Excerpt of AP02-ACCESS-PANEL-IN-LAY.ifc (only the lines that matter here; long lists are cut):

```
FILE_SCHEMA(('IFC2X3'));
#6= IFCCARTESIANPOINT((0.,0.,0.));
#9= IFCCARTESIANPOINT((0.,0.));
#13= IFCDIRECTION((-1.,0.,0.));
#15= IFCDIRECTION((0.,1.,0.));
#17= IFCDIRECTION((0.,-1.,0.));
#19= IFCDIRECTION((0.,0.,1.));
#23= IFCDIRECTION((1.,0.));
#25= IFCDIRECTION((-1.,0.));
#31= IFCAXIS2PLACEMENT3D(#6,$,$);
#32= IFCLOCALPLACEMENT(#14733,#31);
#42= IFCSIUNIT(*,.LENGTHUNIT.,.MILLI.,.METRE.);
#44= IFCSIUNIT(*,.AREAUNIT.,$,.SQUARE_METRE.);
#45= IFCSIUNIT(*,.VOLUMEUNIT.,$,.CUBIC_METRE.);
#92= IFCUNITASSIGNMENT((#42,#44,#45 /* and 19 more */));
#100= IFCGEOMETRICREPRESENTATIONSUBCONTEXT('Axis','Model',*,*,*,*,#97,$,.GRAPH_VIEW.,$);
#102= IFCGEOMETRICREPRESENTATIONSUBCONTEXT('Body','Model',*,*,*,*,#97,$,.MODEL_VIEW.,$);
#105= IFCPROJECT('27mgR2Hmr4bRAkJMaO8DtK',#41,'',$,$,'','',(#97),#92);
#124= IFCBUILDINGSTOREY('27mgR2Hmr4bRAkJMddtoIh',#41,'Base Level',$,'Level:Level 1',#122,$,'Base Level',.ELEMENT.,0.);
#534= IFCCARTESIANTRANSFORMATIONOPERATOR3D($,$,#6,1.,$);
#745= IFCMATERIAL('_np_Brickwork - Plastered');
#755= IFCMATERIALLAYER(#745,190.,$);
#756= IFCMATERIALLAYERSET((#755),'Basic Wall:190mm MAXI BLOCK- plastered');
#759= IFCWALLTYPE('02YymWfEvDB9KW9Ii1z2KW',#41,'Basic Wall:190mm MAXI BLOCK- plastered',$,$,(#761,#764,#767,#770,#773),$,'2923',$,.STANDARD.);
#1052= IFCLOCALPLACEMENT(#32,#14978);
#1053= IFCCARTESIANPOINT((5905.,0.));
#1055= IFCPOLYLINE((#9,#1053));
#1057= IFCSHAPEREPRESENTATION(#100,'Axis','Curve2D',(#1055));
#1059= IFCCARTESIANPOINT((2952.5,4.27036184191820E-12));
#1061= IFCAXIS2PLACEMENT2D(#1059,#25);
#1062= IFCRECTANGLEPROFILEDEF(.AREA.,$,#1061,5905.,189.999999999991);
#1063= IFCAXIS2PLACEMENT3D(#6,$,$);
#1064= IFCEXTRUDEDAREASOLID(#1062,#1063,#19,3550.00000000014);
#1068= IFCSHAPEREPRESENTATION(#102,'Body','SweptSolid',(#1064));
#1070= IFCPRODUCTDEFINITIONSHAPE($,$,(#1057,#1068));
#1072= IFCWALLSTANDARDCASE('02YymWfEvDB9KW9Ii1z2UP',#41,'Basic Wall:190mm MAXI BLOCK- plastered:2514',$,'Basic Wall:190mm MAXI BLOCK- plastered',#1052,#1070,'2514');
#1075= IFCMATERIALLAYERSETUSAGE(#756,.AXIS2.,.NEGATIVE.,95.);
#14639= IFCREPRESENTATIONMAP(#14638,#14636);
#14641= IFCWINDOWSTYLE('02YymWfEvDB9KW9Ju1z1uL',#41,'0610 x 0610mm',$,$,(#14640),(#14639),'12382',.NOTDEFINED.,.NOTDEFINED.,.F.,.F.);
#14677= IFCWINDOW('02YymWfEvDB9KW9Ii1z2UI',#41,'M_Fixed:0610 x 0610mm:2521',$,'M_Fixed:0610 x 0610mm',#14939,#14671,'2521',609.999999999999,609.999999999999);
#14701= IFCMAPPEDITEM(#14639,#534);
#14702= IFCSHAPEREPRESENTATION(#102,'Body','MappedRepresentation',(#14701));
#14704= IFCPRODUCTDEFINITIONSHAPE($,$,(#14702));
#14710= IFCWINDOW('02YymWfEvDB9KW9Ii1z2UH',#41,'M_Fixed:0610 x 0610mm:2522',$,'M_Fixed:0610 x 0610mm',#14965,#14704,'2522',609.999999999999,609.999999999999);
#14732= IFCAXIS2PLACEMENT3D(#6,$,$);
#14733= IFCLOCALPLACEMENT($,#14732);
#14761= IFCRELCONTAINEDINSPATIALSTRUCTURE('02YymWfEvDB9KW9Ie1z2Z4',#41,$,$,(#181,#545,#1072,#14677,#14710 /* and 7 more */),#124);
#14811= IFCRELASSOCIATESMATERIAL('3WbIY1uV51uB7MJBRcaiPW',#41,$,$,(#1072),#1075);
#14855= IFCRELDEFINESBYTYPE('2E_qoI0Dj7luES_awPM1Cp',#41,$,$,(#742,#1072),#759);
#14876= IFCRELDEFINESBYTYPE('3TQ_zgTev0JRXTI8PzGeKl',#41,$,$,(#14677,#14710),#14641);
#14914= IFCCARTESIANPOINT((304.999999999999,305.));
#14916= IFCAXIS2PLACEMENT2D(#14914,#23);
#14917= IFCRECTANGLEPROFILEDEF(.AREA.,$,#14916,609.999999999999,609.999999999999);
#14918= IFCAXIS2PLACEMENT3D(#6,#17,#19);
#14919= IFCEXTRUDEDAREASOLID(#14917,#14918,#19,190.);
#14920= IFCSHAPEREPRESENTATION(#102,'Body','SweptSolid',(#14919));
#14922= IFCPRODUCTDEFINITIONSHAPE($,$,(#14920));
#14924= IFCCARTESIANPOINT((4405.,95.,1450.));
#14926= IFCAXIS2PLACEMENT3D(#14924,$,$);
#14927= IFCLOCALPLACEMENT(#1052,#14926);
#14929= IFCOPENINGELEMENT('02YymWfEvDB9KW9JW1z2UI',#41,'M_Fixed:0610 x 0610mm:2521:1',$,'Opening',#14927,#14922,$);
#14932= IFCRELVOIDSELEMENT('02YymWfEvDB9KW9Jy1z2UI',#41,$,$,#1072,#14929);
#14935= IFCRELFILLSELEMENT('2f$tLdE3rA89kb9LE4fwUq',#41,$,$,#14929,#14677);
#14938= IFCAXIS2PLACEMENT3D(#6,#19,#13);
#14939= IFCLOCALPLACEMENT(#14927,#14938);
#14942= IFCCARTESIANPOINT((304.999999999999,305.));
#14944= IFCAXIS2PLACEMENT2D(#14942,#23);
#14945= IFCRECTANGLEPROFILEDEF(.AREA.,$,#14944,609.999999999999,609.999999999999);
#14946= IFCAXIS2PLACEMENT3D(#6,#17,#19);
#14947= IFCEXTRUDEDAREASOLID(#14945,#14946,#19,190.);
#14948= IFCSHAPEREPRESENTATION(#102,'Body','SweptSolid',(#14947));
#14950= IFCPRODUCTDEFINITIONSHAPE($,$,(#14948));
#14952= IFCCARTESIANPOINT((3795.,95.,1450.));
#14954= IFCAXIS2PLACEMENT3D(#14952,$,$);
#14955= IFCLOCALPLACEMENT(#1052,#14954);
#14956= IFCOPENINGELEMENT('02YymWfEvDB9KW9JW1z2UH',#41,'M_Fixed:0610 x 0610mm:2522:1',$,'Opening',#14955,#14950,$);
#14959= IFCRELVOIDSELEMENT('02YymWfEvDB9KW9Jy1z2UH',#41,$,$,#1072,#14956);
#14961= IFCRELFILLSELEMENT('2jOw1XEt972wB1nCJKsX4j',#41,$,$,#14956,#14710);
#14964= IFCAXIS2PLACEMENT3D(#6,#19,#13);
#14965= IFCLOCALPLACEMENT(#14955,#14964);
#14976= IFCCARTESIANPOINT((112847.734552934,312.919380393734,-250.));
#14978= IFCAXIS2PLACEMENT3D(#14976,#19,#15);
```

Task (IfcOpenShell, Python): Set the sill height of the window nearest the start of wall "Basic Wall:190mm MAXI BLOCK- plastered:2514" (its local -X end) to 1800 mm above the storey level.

```python
import numpy as np
import ifcopenshell
import ifcopenshell.api.geometry
import ifcopenshell.geom
import ifcopenshell.util.element
import ifcopenshell.util.placement
import ifcopenshell.util.shape
import ifcopenshell.util.unit

model = ifcopenshell.open("AP02-ACCESS-PANEL-IN-LAY.ifc")
unit_scale = ifcopenshell.util.unit.calculate_unit_scale(model)

window = model.by_id(14710)
opening = window.FillsVoids[0].RelatingOpeningElement
storey = ifcopenshell.util.element.get_container(window, ifc_class="IfcBuildingStorey")
level = ifcopenshell.util.placement.get_local_placement(storey.ObjectPlacement)[2, 3]

# The opening's origin need not be at the sill, so measure its lowest point.
shape = ifcopenshell.geom.create_shape(ifcopenshell.geom.settings(), opening)
bottom = ifcopenshell.util.shape.get_shape_bottom_elevation(shape, shape.geometry) / unit_scale
dz = level + 1.8 / unit_scale - bottom

shift = np.array([0.0, 0.0, dz])
# The window is placed relative to its opening, so it follows when the opening moves.
matrix = ifcopenshell.util.placement.get_local_placement(opening.ObjectPlacement)
matrix[:3, 3] += shift
ifcopenshell.api.geometry.edit_object_placement(
    model, product=opening, matrix=matrix, is_si=False, should_transform_children=True
)

print(f"moved by {dz * unit_scale:+.3f} m")

model.write("AP02-ACCESS-PANEL-IN-LAY_rev.ifc")
```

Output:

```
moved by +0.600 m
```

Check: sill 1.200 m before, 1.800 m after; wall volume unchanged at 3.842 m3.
